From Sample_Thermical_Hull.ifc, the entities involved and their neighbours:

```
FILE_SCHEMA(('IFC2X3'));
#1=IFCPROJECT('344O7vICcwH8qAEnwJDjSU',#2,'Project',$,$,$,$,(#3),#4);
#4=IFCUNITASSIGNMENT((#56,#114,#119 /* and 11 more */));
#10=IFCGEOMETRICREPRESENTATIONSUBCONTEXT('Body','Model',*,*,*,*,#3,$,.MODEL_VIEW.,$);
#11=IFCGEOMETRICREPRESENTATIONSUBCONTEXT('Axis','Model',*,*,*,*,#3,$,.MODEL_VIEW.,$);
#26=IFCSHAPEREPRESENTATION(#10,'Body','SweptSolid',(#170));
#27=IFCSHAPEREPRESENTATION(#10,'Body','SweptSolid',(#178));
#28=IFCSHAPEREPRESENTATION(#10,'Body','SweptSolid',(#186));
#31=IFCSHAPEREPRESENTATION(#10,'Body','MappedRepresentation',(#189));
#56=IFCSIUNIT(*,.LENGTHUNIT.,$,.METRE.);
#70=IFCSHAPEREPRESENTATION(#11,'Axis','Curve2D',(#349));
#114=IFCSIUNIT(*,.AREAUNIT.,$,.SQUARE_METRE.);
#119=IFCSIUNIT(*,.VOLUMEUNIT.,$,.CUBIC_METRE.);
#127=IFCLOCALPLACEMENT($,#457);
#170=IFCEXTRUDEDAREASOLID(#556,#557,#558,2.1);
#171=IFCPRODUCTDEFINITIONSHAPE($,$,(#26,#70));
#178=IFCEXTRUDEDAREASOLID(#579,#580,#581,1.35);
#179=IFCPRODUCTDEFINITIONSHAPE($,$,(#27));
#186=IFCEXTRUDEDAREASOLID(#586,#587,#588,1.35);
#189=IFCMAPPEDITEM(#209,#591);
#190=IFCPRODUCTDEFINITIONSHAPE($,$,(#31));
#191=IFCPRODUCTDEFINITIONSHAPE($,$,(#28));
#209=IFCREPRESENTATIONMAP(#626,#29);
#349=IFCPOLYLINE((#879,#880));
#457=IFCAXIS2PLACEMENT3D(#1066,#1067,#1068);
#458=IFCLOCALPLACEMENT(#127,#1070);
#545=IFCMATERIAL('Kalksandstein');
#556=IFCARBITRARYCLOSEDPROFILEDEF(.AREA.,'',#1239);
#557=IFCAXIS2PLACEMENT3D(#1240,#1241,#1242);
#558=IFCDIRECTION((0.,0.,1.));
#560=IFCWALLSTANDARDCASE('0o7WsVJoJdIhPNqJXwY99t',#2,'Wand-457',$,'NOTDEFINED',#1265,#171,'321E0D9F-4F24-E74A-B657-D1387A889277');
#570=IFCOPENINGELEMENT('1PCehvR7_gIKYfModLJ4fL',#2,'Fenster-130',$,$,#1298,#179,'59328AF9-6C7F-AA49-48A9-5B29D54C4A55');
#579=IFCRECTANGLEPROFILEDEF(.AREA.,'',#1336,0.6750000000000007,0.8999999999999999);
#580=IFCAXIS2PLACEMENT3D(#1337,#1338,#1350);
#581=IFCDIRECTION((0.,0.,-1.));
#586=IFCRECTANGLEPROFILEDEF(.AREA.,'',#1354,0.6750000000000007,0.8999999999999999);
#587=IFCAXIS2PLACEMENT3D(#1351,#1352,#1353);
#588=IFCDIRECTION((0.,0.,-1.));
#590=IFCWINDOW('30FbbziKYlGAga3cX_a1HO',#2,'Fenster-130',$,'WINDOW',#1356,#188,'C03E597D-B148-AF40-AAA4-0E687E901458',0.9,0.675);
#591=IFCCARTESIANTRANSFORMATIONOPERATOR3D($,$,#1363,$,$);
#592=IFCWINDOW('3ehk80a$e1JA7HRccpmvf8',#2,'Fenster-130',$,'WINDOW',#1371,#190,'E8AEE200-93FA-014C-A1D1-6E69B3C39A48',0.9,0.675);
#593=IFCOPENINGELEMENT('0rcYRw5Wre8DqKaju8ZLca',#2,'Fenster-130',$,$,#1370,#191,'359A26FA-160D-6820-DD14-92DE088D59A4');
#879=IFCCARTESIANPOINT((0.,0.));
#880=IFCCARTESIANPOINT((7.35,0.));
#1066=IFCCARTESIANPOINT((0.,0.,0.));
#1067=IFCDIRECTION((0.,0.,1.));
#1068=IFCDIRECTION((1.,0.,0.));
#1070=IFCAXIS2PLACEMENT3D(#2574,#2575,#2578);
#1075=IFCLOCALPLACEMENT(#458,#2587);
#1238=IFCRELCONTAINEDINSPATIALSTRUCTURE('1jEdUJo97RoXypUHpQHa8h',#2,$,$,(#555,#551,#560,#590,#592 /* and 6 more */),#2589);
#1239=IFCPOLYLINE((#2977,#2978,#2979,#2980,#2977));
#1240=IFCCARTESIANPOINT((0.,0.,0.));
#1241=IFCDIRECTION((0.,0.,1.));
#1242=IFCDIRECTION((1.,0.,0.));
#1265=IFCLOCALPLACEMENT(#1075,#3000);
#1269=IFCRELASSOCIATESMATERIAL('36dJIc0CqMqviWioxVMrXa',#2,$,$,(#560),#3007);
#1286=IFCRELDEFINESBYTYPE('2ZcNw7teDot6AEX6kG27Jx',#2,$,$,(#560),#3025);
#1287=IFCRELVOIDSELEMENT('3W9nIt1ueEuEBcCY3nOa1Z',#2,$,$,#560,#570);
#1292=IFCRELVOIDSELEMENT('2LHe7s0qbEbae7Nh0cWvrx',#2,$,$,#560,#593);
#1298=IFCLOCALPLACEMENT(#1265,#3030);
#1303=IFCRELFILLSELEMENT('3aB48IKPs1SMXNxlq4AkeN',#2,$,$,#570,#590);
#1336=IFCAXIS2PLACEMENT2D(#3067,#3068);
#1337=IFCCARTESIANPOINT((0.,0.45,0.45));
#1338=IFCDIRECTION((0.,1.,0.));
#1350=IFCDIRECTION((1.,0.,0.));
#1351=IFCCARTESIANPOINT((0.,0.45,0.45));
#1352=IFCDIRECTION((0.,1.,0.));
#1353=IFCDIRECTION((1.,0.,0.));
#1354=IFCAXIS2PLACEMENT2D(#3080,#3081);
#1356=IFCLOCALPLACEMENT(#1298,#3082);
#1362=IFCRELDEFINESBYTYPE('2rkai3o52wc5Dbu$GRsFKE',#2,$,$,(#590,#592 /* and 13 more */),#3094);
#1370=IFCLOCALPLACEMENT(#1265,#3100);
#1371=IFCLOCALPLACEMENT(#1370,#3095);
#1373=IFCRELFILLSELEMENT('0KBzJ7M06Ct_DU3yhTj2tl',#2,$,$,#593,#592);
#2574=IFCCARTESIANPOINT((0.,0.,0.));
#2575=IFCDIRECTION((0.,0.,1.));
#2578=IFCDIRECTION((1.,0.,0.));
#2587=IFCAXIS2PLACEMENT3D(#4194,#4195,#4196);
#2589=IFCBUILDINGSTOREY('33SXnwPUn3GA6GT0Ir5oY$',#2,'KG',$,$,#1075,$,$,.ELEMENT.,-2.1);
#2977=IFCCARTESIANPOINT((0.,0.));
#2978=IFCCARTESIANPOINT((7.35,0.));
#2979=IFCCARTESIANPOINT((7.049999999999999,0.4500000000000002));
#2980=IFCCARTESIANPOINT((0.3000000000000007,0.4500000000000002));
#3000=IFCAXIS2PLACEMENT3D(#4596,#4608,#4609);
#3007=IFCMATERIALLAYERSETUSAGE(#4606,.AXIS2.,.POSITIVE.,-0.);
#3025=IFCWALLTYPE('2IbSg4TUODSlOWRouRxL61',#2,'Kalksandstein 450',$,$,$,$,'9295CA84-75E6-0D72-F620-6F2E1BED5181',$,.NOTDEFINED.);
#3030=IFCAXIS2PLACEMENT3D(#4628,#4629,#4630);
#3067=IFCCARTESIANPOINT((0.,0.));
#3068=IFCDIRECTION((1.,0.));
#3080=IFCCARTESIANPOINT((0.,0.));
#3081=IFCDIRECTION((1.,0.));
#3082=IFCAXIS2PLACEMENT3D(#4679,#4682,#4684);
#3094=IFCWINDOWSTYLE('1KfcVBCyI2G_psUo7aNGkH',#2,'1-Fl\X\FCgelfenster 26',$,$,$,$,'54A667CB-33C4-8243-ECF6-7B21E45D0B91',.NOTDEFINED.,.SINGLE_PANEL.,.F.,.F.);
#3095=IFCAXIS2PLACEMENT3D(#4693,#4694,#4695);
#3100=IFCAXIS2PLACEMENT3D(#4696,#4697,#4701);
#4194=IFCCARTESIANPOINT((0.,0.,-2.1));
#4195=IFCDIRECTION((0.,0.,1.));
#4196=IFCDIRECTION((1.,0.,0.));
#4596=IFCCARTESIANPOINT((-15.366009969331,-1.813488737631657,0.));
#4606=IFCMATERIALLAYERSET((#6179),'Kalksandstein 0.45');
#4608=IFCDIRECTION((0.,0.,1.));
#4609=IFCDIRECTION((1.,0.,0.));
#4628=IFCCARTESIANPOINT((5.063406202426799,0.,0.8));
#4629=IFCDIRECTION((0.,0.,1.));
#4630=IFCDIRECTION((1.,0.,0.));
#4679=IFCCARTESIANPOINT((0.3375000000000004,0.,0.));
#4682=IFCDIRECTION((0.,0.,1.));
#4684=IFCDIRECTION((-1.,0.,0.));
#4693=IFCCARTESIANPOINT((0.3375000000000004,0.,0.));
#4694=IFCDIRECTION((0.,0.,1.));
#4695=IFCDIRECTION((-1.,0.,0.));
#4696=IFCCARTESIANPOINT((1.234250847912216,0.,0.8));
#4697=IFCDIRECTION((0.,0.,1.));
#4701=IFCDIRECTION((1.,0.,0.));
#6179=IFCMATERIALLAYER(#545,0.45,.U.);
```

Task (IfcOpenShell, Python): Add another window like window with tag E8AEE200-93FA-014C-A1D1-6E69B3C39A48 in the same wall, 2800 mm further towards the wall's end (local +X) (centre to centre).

```python
import ifcopenshell
import ifcopenshell.api.feature
import ifcopenshell.api.geometry
import ifcopenshell.api.root
import ifcopenshell.geom
import ifcopenshell.util.element
import ifcopenshell.util.placement
import ifcopenshell.util.shape
import ifcopenshell.util.unit

model = ifcopenshell.open("Sample_Thermical_Hull.ifc")
unit_scale = ifcopenshell.util.unit.calculate_unit_scale(model)
settings = ifcopenshell.geom.settings()


def volume(element):
    """Net volume in cubic metres, openings subtracted."""
    shape = ifcopenshell.geom.create_shape(settings, element)
    return ifcopenshell.util.shape.get_volume(shape.geometry)


def reuse_history(source, copy):
    """copy_class also copies each property set's owner history, people and application; keep the originals."""
    for rel in copy.IsDefinedBy:
        if rel.is_a("IfcRelDefinesByProperties") and (history := rel.RelatingPropertyDefinition.OwnerHistory):
            rel.RelatingPropertyDefinition.OwnerHistory = source.OwnerHistory
            ifcopenshell.util.element.remove_deep2(model, history)


window = model.by_guid("3ehk80a$e1JA7HRccpmvf8")
opening = window.FillsVoids[0].RelatingOpeningElement
wall = opening.VoidsElements[0].RelatingBuildingElement
before = volume(wall)
shift = ifcopenshell.util.placement.get_local_placement(wall.ObjectPlacement)[:3, 0] * 2.8 / unit_scale

# copy_class copies the void relationship, type, container and properties, but no geometry.
new_opening = ifcopenshell.api.root.copy_class(model, product=opening)
new_opening.Representation = ifcopenshell.util.element.copy_deep(
    model, opening.Representation, exclude=["IfcGeometricRepresentationContext", "IfcRepresentationMap"]
)
new_opening.Tag = None
new_window = ifcopenshell.api.root.copy_class(model, product=window)
new_window.Representation = ifcopenshell.util.element.copy_deep(
    model, window.Representation, exclude=["IfcGeometricRepresentationContext", "IfcRepresentationMap"]
)
new_window.Tag = None
reuse_history(window, new_window)
fills = ifcopenshell.api.feature.add_filling(model, opening=new_opening, element=new_window)
fills.OwnerHistory = new_window.OwnerHistory  # required in IFC2X3

for old, new in ((opening, new_opening), (window, new_window)):
    matrix = ifcopenshell.util.placement.get_local_placement(old.ObjectPlacement)
    matrix[:3, 3] += shift
    ifcopenshell.api.geometry.edit_object_placement(model, product=new, matrix=matrix, is_si=False)

after = volume(wall)

print(f"wall volume {before:.3f} -> {after:.3f} m3")

model.write("Sample_Thermical_Hull_updated.ifc")
```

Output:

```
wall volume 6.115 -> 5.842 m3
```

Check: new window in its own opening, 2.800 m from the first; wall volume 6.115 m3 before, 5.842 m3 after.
